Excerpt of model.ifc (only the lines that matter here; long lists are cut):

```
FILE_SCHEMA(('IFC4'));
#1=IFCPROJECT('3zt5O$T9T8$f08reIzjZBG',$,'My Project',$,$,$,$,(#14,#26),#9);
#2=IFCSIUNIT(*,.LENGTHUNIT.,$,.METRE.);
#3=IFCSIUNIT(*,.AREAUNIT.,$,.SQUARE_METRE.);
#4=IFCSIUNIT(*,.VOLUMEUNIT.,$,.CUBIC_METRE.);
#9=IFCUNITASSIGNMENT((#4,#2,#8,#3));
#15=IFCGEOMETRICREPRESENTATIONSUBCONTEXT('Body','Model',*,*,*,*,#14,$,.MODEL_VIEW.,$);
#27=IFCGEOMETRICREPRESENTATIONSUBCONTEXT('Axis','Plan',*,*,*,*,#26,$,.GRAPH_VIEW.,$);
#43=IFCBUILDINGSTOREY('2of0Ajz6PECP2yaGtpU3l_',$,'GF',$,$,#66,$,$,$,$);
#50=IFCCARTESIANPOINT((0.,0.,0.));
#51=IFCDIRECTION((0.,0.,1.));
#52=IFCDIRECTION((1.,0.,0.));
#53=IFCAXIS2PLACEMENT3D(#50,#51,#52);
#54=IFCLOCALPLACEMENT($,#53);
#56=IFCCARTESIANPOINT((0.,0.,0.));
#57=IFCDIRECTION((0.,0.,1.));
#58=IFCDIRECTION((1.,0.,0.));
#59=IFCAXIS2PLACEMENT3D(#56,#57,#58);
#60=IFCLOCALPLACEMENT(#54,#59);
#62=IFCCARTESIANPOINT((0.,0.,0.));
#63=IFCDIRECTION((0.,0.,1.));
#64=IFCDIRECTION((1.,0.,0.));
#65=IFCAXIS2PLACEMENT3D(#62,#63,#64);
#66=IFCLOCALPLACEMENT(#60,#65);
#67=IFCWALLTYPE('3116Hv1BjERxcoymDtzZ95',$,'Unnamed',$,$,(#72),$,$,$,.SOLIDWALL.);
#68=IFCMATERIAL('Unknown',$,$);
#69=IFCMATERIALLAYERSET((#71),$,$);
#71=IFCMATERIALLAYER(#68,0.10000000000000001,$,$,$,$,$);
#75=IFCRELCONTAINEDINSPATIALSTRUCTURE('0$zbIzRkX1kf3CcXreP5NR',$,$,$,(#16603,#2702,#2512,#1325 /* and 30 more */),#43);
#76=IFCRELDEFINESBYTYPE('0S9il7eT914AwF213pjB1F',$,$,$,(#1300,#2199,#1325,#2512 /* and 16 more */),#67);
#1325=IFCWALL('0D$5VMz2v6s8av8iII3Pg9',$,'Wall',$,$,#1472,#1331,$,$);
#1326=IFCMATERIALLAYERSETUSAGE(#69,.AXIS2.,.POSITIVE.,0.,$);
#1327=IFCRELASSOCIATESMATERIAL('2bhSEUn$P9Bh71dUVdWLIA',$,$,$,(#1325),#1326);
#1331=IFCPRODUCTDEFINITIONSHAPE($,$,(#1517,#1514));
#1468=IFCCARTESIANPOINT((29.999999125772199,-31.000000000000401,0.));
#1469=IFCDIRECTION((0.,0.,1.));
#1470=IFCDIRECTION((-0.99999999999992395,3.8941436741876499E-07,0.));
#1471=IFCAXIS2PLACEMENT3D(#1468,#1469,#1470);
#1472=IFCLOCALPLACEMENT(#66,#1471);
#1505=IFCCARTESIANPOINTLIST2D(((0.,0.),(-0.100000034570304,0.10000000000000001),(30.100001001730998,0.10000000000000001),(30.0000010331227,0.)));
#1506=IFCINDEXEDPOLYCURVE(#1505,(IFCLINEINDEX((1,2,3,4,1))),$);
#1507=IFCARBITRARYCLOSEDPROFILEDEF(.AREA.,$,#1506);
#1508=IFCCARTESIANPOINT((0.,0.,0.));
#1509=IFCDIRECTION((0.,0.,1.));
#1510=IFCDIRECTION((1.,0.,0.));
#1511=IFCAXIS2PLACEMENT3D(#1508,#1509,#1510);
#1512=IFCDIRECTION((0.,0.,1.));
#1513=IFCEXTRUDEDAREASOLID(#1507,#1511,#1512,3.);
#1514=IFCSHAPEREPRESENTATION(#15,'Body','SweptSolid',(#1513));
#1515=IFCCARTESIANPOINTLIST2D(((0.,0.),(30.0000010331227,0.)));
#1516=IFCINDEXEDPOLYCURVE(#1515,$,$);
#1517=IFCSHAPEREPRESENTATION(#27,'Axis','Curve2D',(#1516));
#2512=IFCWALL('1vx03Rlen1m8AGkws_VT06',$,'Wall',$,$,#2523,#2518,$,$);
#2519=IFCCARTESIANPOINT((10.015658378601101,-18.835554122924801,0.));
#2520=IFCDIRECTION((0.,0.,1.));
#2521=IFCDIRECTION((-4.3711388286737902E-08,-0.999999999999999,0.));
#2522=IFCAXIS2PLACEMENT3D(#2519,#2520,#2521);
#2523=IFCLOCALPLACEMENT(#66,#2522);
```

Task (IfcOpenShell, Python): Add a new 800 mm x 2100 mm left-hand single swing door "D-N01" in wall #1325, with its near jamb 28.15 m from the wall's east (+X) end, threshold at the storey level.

```python
import numpy as np
import ifcopenshell
import ifcopenshell.api.feature
import ifcopenshell.api.geometry
import ifcopenshell.api.root
import ifcopenshell.api.spatial
import ifcopenshell.geom
import ifcopenshell.util.element
import ifcopenshell.util.placement
import ifcopenshell.util.representation
import ifcopenshell.util.shape
import ifcopenshell.util.unit

model = ifcopenshell.open("model.ifc")
unit_scale = ifcopenshell.util.unit.calculate_unit_scale(model)
settings = ifcopenshell.geom.settings()


def volume(element):
    """Net volume in cubic metres, openings subtracted."""
    shape = ifcopenshell.geom.create_shape(settings, element)
    return ifcopenshell.util.shape.get_volume(shape.geometry)


wall = model.by_guid("0D$5VMz2v6s8av8iII3Pg9")
storey = ifcopenshell.util.element.get_container(wall, ifc_class="IfcBuildingStorey")
context = ifcopenshell.util.representation.get_context(model, "Model", "Body", "MODEL_VIEW")
before = volume(wall)

width, height, from_end, sill = 0.8, 2.1, 28.15, 0.0  # metres

# The wall runs along its own X axis, and the end named is its -X end.
wall_shape = ifcopenshell.geom.create_shape(settings, wall)
x, y, z = ifcopenshell.util.shape.get_vertices(wall_shape.geometry).T
start = x.min() + from_end
face, thickness = float(y.min()), float(y.max() - y.min())
wall_matrix = ifcopenshell.util.placement.get_local_placement(wall.ObjectPlacement)
level = ifcopenshell.util.placement.get_local_placement(storey.ObjectPlacement)[2, 3]


def in_wall(x, y):
    """Placement at x, y metres in the wall's axes, at sill height."""
    matrix = wall_matrix.copy()
    matrix[:, 3] = wall_matrix @ np.array([x / unit_scale, y / unit_scale, 0.0, 1.0])
    matrix[2, 3] = level + sill / unit_scale
    return matrix


# Opening: a box that overshoots both wall faces by 50 mm.
opening = ifcopenshell.api.root.create_entity(model, ifc_class="IfcOpeningElement", predefined_type="OPENING")
box = ifcopenshell.api.geometry.add_wall_representation(
    model, context=context, length=width, height=height, thickness=thickness + 0.1
)
ifcopenshell.api.geometry.assign_representation(model, product=opening, representation=box)
ifcopenshell.api.geometry.edit_object_placement(model, product=opening, matrix=in_wall(start, face - 0.05), is_si=False)
ifcopenshell.api.feature.add_feature(model, feature=opening, element=wall)

door = ifcopenshell.api.root.create_entity(model, ifc_class="IfcDoor", name="D-N01", predefined_type="DOOR")
door.OverallWidth, door.OverallHeight = width / unit_scale, height / unit_scale
door.OperationType = "SINGLE_SWING_LEFT"
body = ifcopenshell.api.geometry.add_door_representation(
    model,
    context=context,
    overall_width=door.OverallWidth,
    overall_height=door.OverallHeight,
    operation_type="SINGLE_SWING_LEFT",
    lining_properties={"LiningDepth": thickness / unit_scale, "ThresholdDepth": thickness / unit_scale},
)
ifcopenshell.api.geometry.assign_representation(model, product=door, representation=body)
ifcopenshell.api.spatial.assign_container(model, products=[door], relating_structure=storey)
ifcopenshell.api.feature.add_filling(model, opening=opening, element=door)

# The lining spans the wall, so the door starts at the wall face.
ifcopenshell.api.geometry.edit_object_placement(model, product=door, matrix=in_wall(start, face), is_si=False)

after = volume(wall)

print(f"wall volume {before:.3f} -> {after:.3f} m3")

model.write("model_rev.ifc")
```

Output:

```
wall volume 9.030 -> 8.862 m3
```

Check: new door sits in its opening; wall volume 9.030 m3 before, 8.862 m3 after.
